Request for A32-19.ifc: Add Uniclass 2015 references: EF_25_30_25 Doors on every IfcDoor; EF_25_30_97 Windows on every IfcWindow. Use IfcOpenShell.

First a look at what the model holds.

```python
import ifcopenshell

model = ifcopenshell.open("A32-19.ifc")
print(model.schema)
print("classifications:", [c.Name for c in model.by_type("IfcClassification")])
for ifc_class in ("IfcDoor", "IfcRoof", "IfcStair", "IfcWall", "IfcWindow"):
    print(ifc_class, len(model.by_type(ifc_class)))
```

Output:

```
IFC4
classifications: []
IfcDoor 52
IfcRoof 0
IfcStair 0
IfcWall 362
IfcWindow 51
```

```python
import ifcopenshell
import ifcopenshell.api.classification

model = ifcopenshell.open("A32-19.ifc")

system = ifcopenshell.api.classification.add_classification(model, classification="Uniclass 2015")

codes = {
    "IfcDoor": ("EF_25_30_25", "Doors"),
    "IfcWindow": ("EF_25_30_97", "Windows"),
}
for ifc_class, (code, name) in codes.items():
    products = model.by_type(ifc_class)
    ifcopenshell.api.classification.add_reference(
        model, products=products, classification=system, identification=code, name=name
    )
    print(code, len(products))

model.write("A32-19_edited.ifc")
```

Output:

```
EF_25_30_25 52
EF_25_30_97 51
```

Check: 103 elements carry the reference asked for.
